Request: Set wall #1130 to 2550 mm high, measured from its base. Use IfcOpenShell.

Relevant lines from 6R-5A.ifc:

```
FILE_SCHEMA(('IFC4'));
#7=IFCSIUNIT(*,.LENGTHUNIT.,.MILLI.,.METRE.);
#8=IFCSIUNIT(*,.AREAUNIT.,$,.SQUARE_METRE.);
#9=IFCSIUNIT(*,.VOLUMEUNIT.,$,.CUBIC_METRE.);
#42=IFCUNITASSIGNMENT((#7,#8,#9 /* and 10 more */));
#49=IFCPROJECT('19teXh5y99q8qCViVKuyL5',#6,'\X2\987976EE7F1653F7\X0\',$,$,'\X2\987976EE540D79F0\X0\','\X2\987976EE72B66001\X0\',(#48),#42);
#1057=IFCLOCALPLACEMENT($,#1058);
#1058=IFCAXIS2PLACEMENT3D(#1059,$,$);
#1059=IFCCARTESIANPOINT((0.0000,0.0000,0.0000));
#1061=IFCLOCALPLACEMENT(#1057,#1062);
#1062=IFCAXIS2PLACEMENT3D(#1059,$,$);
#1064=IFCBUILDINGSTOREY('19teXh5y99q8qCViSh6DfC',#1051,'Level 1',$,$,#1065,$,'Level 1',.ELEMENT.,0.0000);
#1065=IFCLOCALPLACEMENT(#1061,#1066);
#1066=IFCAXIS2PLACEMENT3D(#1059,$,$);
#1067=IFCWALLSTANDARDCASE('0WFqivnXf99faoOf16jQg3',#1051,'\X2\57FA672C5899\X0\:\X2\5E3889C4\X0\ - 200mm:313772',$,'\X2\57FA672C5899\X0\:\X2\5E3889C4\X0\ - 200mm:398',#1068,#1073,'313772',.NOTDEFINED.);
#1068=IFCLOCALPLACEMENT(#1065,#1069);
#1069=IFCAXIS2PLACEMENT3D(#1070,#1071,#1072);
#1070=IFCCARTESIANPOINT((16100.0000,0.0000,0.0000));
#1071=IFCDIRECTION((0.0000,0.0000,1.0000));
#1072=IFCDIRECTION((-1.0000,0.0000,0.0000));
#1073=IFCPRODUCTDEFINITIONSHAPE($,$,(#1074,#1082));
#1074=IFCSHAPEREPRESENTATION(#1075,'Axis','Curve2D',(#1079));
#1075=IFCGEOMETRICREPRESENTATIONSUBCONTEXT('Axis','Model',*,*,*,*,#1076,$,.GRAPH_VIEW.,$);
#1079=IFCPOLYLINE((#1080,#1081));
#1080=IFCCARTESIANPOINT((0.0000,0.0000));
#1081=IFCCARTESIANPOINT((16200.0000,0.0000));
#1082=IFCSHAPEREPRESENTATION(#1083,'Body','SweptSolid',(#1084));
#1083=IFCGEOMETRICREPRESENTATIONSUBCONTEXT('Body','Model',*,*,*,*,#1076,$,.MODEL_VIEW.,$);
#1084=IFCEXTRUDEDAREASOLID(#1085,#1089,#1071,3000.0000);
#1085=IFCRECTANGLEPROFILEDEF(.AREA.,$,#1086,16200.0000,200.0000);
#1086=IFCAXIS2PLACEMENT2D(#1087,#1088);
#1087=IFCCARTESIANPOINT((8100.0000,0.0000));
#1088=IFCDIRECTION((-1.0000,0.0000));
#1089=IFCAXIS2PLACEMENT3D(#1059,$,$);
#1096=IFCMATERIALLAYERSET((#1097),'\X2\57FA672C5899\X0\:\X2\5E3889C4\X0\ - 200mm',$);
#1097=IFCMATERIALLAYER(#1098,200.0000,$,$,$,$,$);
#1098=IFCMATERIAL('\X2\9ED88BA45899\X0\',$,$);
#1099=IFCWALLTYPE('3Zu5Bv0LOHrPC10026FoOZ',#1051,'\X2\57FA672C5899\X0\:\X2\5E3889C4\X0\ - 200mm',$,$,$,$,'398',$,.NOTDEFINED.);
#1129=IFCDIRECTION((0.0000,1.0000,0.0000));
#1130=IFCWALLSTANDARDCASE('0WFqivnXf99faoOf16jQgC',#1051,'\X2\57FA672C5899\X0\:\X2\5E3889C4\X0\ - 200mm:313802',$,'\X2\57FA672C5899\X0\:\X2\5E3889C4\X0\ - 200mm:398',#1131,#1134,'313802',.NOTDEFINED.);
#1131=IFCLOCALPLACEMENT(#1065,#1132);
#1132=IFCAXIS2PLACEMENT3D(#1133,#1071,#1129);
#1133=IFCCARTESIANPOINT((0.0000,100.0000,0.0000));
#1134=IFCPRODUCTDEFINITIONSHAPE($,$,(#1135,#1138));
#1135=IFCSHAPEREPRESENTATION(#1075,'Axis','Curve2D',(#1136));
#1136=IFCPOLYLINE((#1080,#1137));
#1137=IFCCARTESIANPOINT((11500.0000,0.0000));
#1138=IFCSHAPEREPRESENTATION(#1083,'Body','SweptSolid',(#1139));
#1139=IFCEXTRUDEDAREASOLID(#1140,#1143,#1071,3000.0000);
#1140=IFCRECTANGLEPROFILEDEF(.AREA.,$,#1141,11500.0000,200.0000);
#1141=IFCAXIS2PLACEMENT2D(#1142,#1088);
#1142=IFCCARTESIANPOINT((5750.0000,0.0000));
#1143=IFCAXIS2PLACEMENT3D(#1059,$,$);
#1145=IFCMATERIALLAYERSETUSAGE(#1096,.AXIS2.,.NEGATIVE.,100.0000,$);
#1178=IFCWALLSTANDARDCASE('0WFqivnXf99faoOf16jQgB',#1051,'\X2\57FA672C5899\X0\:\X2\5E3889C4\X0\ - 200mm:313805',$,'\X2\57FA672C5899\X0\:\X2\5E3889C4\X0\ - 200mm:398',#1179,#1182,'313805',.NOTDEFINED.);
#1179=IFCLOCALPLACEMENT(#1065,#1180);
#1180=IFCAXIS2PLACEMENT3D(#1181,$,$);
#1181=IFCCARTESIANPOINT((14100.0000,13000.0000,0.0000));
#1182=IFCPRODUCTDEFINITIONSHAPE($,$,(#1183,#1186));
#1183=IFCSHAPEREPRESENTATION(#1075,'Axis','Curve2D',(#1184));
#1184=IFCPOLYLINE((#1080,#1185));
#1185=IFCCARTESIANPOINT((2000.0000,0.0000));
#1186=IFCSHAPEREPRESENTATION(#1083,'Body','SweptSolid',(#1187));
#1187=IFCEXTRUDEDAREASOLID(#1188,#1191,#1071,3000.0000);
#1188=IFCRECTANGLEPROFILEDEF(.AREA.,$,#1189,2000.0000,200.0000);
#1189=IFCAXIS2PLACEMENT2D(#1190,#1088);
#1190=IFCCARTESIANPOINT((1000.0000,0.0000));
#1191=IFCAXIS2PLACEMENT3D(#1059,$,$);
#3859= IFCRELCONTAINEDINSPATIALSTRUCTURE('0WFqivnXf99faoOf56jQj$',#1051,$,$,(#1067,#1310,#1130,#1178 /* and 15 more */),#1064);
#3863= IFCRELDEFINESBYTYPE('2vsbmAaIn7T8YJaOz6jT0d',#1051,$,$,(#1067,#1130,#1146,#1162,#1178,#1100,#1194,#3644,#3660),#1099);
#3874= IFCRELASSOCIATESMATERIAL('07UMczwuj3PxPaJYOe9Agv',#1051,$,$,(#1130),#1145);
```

```python
import ifcopenshell
import ifcopenshell.geom
import ifcopenshell.util.representation
import ifcopenshell.util.shape
import ifcopenshell.util.unit

model = ifcopenshell.open("6R-5A.ifc")
unit_scale = ifcopenshell.util.unit.calculate_unit_scale(model)
settings = ifcopenshell.geom.settings()


def volume(element):
    """Net volume in cubic metres, openings subtracted."""
    shape = ifcopenshell.geom.create_shape(settings, element)
    return ifcopenshell.util.shape.get_volume(shape.geometry)


wall = model.by_id(1130)
before = volume(wall)

body = ifcopenshell.util.representation.get_representation(wall, "Model", "Body")
solid = body.Items[0]
old_height = solid.Depth
solid.Depth = 2.55 / unit_scale
after = volume(wall)

print(f"height {old_height:g} -> {solid.Depth:g}, volume {before:.3f} -> {after:.3f} m3")

model.write("6R-5A-out.ifc")
```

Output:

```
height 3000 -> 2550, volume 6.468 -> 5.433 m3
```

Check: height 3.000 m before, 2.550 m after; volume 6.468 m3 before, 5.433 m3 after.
